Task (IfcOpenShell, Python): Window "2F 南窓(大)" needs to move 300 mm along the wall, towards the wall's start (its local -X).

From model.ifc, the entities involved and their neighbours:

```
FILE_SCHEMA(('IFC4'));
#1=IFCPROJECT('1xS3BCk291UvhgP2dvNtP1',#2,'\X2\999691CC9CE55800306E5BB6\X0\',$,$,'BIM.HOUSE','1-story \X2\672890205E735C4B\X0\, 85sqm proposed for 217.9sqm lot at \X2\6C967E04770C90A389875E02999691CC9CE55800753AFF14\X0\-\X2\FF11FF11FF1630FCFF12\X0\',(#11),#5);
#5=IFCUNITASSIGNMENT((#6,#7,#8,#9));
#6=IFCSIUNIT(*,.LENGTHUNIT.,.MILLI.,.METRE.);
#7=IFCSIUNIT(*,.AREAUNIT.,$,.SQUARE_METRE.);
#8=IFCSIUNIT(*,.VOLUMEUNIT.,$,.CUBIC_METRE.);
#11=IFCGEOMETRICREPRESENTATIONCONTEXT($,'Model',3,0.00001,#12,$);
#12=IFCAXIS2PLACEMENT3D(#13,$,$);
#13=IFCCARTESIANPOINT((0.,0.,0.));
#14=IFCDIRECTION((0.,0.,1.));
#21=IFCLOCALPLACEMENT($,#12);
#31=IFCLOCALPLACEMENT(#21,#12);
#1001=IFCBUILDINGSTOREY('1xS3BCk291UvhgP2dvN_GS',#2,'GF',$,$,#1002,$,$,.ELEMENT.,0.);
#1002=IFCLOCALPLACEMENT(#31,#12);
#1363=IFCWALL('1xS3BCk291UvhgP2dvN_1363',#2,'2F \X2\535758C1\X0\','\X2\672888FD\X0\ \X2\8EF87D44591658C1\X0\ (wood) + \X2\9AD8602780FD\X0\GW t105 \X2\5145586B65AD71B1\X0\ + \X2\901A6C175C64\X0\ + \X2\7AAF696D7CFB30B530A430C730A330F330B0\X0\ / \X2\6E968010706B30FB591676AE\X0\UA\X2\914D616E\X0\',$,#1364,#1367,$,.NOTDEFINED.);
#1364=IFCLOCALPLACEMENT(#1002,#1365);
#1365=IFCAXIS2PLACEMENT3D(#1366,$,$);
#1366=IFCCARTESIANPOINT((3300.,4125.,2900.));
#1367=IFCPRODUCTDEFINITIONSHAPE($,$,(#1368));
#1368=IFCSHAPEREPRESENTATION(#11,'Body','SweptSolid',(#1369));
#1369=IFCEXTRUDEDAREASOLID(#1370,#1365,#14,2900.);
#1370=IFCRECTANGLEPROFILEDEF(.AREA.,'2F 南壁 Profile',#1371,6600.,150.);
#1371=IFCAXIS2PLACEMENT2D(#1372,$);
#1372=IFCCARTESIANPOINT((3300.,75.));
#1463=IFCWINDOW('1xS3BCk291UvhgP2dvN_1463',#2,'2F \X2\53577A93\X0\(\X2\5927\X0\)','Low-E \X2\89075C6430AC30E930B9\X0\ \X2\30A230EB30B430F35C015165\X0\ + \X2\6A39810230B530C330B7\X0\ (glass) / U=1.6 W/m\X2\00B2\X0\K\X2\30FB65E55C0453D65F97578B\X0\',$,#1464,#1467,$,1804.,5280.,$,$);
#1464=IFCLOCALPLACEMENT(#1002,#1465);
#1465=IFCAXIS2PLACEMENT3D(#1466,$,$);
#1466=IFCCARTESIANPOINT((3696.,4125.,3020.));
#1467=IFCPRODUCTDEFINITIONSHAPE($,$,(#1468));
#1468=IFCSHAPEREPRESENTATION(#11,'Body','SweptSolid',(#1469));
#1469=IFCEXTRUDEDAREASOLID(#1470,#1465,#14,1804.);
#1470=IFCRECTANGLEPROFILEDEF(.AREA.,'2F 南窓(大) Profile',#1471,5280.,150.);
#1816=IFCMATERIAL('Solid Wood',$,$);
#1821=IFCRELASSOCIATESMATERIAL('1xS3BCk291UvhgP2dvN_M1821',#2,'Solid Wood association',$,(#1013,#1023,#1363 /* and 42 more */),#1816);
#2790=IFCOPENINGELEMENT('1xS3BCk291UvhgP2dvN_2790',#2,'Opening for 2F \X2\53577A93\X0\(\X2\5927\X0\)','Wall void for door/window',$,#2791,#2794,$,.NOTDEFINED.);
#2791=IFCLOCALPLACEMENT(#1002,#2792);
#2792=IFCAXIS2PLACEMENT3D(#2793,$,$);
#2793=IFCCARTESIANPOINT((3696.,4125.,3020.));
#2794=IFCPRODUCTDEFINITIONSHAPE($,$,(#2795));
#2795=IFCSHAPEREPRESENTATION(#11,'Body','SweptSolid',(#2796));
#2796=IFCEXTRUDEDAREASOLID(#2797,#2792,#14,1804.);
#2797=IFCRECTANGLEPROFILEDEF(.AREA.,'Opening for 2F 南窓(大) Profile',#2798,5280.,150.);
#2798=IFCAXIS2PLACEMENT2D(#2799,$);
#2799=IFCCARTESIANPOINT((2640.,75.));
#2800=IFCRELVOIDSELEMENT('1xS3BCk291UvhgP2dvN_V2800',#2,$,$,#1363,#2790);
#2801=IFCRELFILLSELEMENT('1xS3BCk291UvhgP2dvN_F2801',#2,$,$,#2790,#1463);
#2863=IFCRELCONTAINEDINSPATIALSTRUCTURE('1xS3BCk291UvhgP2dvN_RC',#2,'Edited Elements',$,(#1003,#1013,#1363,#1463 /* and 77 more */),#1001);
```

```python
import ifcopenshell
import ifcopenshell.api.geometry
import ifcopenshell.util.placement

model = ifcopenshell.open("model.ifc")

window = model.by_guid("1xS3BCk291UvhgP2dvN_1463")
opening = window.FillsVoids[0].RelatingOpeningElement
wall = opening.VoidsElements[0].RelatingBuildingElement

wall_matrix = ifcopenshell.util.placement.get_local_placement(wall.ObjectPlacement)
shift = wall_matrix[:3, 0] * -300.0
before = ifcopenshell.util.placement.get_local_placement(window.ObjectPlacement)[:3, 3].copy()

# The window is not placed relative to its opening, so move both.
for product in (opening, window):
    matrix = ifcopenshell.util.placement.get_local_placement(product.ObjectPlacement)
    matrix[:3, 3] += shift
    ifcopenshell.api.geometry.edit_object_placement(model, product=product, matrix=matrix, is_si=False)

after = ifcopenshell.util.placement.get_local_placement(window.ObjectPlacement)[:3, 3]
print("window moved by", (after - before).round(3) + 0.0)

model.write("model_edited.ifc")
```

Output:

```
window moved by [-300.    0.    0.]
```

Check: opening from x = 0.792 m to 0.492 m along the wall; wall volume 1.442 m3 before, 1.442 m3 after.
